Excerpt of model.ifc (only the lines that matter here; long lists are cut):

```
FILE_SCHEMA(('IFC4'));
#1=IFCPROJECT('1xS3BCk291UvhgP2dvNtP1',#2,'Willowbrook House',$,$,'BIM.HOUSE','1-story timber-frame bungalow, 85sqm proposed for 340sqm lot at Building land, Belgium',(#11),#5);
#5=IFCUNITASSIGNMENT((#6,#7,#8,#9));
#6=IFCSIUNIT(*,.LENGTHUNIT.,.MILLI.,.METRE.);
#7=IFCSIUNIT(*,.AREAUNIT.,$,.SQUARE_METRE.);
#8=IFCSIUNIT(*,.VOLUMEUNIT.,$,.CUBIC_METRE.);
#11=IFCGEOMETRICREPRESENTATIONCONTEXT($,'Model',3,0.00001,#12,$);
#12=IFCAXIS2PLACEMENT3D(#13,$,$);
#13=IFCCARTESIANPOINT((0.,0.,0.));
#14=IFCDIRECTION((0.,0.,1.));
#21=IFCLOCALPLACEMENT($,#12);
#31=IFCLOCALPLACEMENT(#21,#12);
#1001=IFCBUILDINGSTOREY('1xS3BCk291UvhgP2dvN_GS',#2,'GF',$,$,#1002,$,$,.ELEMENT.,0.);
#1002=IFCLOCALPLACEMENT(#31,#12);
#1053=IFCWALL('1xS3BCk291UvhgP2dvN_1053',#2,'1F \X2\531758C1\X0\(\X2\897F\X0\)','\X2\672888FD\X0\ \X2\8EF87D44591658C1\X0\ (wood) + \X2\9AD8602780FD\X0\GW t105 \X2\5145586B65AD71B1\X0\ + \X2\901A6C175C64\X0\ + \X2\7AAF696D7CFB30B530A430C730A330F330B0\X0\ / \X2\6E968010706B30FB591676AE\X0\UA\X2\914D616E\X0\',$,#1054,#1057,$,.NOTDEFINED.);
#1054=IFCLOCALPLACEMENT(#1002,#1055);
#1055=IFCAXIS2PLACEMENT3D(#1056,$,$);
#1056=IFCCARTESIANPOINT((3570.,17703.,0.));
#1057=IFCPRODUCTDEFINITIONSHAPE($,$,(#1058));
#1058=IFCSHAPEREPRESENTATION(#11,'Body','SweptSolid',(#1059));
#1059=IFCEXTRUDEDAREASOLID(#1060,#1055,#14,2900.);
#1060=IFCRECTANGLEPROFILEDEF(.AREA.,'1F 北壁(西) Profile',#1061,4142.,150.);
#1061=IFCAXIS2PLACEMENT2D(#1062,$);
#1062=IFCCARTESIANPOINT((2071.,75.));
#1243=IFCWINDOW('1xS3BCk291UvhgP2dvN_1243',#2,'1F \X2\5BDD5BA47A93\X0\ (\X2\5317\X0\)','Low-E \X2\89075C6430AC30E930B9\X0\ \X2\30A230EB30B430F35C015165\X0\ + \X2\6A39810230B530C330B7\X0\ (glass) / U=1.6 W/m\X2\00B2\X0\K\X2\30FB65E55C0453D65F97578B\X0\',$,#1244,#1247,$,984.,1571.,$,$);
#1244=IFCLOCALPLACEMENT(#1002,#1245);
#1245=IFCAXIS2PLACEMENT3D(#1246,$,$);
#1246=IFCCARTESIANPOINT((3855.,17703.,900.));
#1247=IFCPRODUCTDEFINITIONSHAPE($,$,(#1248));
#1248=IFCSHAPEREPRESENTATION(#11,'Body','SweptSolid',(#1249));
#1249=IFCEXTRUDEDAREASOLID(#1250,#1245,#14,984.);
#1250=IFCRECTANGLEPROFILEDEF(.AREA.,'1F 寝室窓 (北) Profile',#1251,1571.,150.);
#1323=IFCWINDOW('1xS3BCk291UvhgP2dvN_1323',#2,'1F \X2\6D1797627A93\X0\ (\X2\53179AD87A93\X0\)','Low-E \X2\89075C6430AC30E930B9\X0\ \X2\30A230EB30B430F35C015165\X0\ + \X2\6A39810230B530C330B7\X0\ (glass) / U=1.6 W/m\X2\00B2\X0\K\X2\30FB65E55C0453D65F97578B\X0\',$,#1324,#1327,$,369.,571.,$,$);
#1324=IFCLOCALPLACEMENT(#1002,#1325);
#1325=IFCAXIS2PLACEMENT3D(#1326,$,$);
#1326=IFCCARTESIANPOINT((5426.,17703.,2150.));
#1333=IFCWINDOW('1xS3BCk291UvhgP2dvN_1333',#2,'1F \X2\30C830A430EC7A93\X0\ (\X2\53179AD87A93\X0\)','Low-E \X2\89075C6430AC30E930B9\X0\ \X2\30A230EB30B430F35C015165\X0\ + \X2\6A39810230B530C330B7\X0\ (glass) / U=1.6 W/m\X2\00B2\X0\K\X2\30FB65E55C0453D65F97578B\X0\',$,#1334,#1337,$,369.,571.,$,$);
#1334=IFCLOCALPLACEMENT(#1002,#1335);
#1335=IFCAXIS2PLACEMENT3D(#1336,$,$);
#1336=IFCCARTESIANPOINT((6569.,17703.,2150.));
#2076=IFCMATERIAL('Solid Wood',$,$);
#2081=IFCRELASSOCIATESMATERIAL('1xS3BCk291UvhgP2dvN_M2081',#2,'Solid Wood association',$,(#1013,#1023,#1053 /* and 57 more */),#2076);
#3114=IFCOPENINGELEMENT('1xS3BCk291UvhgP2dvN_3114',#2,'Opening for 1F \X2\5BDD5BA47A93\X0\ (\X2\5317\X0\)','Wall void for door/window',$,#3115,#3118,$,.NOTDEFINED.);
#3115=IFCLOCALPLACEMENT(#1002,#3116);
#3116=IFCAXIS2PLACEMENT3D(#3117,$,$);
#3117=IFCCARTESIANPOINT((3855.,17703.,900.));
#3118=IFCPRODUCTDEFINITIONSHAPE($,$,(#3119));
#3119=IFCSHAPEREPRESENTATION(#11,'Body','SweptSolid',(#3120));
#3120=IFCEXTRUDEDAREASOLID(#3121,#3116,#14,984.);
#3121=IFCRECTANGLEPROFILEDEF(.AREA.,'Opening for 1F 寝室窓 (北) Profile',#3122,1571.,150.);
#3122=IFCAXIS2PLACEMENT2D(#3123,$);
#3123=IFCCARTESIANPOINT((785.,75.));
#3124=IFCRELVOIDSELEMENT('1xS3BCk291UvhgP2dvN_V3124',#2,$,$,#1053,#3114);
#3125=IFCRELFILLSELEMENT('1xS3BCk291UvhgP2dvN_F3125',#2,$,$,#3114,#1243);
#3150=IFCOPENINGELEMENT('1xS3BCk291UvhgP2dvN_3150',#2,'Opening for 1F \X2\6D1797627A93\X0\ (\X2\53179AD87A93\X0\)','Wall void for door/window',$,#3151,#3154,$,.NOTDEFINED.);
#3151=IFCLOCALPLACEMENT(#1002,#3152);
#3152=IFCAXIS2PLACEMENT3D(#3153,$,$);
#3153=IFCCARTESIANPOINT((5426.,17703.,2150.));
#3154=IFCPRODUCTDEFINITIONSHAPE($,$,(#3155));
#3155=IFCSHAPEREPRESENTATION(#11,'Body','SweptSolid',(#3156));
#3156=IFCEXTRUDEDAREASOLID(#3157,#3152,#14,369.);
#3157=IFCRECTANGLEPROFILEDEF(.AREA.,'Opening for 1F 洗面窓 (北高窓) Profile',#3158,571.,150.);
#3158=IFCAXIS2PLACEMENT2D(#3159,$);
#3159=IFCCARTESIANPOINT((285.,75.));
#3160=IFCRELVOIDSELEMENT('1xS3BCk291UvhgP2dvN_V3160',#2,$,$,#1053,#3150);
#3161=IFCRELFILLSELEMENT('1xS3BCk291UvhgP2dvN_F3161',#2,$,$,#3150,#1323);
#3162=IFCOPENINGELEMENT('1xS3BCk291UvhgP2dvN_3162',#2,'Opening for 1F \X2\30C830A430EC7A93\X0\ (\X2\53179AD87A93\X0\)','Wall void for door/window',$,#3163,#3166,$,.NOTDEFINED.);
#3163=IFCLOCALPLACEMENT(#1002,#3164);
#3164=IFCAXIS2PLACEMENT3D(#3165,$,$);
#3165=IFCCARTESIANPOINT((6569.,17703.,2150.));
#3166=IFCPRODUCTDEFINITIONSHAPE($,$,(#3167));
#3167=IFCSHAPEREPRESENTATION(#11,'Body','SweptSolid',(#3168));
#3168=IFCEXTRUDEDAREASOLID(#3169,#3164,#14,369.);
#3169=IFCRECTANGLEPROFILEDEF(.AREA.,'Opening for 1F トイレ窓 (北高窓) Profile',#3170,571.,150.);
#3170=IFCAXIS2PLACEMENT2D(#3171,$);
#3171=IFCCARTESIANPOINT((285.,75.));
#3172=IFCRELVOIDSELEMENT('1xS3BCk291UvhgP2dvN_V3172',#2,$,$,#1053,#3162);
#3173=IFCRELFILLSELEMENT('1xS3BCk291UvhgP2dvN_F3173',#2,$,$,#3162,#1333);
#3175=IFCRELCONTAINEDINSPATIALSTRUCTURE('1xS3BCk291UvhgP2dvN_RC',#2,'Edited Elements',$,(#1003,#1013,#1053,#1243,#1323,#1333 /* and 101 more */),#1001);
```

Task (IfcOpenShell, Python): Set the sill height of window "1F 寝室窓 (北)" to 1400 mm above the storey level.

```python
import numpy as np
import ifcopenshell
import ifcopenshell.api.geometry
import ifcopenshell.geom
import ifcopenshell.util.element
import ifcopenshell.util.placement
import ifcopenshell.util.shape
import ifcopenshell.util.unit

model = ifcopenshell.open("model.ifc")
unit_scale = ifcopenshell.util.unit.calculate_unit_scale(model)

window = model.by_guid("1xS3BCk291UvhgP2dvN_1243")
opening = window.FillsVoids[0].RelatingOpeningElement
storey = ifcopenshell.util.element.get_container(window, ifc_class="IfcBuildingStorey")
level = ifcopenshell.util.placement.get_local_placement(storey.ObjectPlacement)[2, 3]

# The opening's origin need not be at the sill, so measure its lowest point.
shape = ifcopenshell.geom.create_shape(ifcopenshell.geom.settings(), opening)
bottom = ifcopenshell.util.shape.get_shape_bottom_elevation(shape, shape.geometry) / unit_scale
dz = level + 1.4 / unit_scale - bottom

shift = np.array([0.0, 0.0, dz])
# The window is not placed relative to its opening, so move both.
for product in (opening, window):
    matrix = ifcopenshell.util.placement.get_local_placement(product.ObjectPlacement)
    matrix[:3, 3] += shift
    ifcopenshell.api.geometry.edit_object_placement(model, product=product, matrix=matrix, is_si=False)

print(f"moved by {dz * unit_scale:+.3f} m")

model.write("model_rev.ifc")
```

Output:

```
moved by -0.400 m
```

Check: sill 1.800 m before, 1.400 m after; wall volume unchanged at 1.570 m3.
